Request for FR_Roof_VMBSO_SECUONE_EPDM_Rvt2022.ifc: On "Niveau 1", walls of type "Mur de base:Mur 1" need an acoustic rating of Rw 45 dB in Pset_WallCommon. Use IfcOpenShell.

First a look at what the model holds.

```python
import ifcopenshell
import ifcopenshell.util.element

model = ifcopenshell.open("FR_Roof_VMBSO_SECUONE_EPDM_Rvt2022.ifc")
print(model.schema)
storey = next(s for s in model.by_type("IfcBuildingStorey") if s.Name == "Niveau 1")
walls = [e for e in ifcopenshell.util.element.get_decomposition(storey) if e.is_a("IfcWall")]
seen = {}
for e in walls:
    element_type = ifcopenshell.util.element.get_type(e)
    key = (element_type.Name if element_type != e and element_type else None, ifcopenshell.util.element.get_pset(e, "Pset_WallCommon", "AcousticRating"))
    seen[key] = seen.get(key, 0) + 1
for (name, value), count in sorted(seen.items(), key=str):
    print(count, "x", name, "|", value)
```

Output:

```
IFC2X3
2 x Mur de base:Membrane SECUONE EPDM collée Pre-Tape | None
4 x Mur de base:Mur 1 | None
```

```python
import ifcopenshell
import ifcopenshell.api.pset
import ifcopenshell.util.element

model = ifcopenshell.open("FR_Roof_VMBSO_SECUONE_EPDM_Rvt2022.ifc")

storey = next(s for s in model.by_type("IfcBuildingStorey") if s.Name == "Niveau 1")
walls = [e for e in ifcopenshell.util.element.get_decomposition(storey) if e.is_a("IfcWall")]

count = 0
for e in walls:
    element_type = ifcopenshell.util.element.get_type(e)
    if element_type in (None, e) or element_type.Name != "Mur de base:Mur 1":
        continue
    # add_pset returns the element's existing set when there is one.
    pset = ifcopenshell.api.pset.add_pset(model, product=e, name="Pset_WallCommon")
    ifcopenshell.api.pset.edit_pset(model, pset=pset, properties={"AcousticRating": "Rw 45 dB"})
    count += 1

print(count, "walls updated")

model.write("FR_Roof_VMBSO_SECUONE_EPDM_Rvt2022_v2.ifc")
```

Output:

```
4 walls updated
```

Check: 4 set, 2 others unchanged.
